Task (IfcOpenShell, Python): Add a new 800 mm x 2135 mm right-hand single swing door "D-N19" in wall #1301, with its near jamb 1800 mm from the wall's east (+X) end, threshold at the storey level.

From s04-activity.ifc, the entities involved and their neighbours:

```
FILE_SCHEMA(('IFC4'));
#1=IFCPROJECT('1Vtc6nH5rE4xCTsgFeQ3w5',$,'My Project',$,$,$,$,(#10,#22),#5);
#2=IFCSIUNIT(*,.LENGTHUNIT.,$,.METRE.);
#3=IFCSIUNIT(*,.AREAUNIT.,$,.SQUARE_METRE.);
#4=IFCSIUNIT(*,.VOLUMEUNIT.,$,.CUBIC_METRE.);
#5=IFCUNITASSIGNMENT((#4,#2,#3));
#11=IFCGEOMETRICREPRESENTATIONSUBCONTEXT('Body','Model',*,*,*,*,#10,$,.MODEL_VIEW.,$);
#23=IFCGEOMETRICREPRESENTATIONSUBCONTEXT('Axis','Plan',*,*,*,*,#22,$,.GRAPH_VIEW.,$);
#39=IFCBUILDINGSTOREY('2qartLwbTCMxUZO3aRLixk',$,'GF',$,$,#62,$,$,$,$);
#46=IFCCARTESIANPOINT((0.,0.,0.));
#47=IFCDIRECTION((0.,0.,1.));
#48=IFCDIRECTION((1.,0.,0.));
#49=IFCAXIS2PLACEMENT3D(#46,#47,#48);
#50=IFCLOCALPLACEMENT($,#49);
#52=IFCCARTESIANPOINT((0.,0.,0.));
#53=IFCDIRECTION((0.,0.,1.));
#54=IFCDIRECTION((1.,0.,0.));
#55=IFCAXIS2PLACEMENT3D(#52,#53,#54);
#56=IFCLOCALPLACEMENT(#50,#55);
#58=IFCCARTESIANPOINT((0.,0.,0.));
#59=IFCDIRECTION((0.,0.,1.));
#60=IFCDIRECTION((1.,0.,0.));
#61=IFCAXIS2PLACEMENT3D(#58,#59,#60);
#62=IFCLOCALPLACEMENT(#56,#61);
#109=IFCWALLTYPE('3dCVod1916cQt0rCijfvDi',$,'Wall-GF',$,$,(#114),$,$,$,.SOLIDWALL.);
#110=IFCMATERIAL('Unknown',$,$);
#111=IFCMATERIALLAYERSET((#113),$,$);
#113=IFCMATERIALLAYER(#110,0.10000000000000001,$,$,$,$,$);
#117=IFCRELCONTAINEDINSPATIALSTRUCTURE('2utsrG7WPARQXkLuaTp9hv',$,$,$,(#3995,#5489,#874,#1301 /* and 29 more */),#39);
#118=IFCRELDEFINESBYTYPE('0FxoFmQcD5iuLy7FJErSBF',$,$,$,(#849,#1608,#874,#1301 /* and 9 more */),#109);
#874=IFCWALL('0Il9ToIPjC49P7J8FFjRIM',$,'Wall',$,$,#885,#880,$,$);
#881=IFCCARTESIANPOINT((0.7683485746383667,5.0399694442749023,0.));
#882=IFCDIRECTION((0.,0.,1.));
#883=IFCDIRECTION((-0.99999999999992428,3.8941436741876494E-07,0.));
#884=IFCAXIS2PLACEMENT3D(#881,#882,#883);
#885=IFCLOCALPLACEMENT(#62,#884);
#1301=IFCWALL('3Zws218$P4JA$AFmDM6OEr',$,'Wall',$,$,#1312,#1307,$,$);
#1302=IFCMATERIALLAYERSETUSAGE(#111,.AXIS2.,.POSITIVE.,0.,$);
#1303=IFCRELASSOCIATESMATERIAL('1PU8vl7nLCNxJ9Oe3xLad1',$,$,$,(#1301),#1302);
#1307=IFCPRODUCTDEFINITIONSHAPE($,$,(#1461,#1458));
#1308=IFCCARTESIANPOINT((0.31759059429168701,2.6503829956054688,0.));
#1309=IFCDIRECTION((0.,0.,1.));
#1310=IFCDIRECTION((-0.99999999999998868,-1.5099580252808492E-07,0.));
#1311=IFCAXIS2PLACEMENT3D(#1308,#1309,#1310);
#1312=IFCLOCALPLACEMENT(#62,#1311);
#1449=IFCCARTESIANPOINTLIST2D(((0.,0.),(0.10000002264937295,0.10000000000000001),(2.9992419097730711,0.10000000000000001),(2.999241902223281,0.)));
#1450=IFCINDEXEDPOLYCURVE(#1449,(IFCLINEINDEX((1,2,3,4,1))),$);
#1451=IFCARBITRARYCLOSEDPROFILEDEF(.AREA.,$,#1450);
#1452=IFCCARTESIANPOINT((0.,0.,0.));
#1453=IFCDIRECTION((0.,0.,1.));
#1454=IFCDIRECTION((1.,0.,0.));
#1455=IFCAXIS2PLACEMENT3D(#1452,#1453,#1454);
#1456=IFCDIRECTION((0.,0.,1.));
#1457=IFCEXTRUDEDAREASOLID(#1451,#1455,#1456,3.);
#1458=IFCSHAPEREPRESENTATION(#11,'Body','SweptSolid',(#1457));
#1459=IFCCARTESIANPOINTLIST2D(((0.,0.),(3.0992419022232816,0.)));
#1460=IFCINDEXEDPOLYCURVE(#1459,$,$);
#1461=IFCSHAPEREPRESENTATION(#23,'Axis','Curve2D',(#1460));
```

```python
import numpy as np
import ifcopenshell
import ifcopenshell.api.feature
import ifcopenshell.api.geometry
import ifcopenshell.api.root
import ifcopenshell.api.spatial
import ifcopenshell.geom
import ifcopenshell.util.element
import ifcopenshell.util.placement
import ifcopenshell.util.representation
import ifcopenshell.util.shape
import ifcopenshell.util.unit

model = ifcopenshell.open("s04-activity.ifc")
unit_scale = ifcopenshell.util.unit.calculate_unit_scale(model)
settings = ifcopenshell.geom.settings()


def volume(element):
    """Net volume in cubic metres, openings subtracted."""
    shape = ifcopenshell.geom.create_shape(settings, element)
    return ifcopenshell.util.shape.get_volume(shape.geometry)


wall = model.by_guid("3Zws218$P4JA$AFmDM6OEr")
storey = ifcopenshell.util.element.get_container(wall, ifc_class="IfcBuildingStorey")
context = ifcopenshell.util.representation.get_context(model, "Model", "Body", "MODEL_VIEW")
before = volume(wall)

width, height, from_end, sill = 0.8, 2.135, 1.8, 0.0  # metres

# The wall runs along its own X axis, and the end named is its -X end.
wall_shape = ifcopenshell.geom.create_shape(settings, wall)
x, y, z = ifcopenshell.util.shape.get_vertices(wall_shape.geometry).T
start = x.min() + from_end
face, thickness = float(y.min()), float(y.max() - y.min())
wall_matrix = ifcopenshell.util.placement.get_local_placement(wall.ObjectPlacement)
level = ifcopenshell.util.placement.get_local_placement(storey.ObjectPlacement)[2, 3]


def in_wall(x, y):
    """Placement at x, y metres in the wall's axes, at sill height."""
    matrix = wall_matrix.copy()
    matrix[:, 3] = wall_matrix @ np.array([x / unit_scale, y / unit_scale, 0.0, 1.0])
    matrix[2, 3] = level + sill / unit_scale
    return matrix


# Opening: a box that overshoots both wall faces by 50 mm.
opening = ifcopenshell.api.root.create_entity(model, ifc_class="IfcOpeningElement", predefined_type="OPENING")
box = ifcopenshell.api.geometry.add_wall_representation(
    model, context=context, length=width, height=height, thickness=thickness + 0.1
)
ifcopenshell.api.geometry.assign_representation(model, product=opening, representation=box)
ifcopenshell.api.geometry.edit_object_placement(model, product=opening, matrix=in_wall(start, face - 0.05), is_si=False)
ifcopenshell.api.feature.add_feature(model, feature=opening, element=wall)

door = ifcopenshell.api.root.create_entity(model, ifc_class="IfcDoor", name="D-N19", predefined_type="DOOR")
door.OverallWidth, door.OverallHeight = width / unit_scale, height / unit_scale
door.OperationType = "SINGLE_SWING_RIGHT"
body = ifcopenshell.api.geometry.add_door_representation(
    model,
    context=context,
    overall_width=door.OverallWidth,
    overall_height=door.OverallHeight,
    operation_type="SINGLE_SWING_RIGHT",
    lining_properties={"LiningDepth": thickness / unit_scale, "ThresholdDepth": thickness / unit_scale},
)
ifcopenshell.api.geometry.assign_representation(model, product=door, representation=body)
ifcopenshell.api.spatial.assign_container(model, products=[door], relating_structure=storey)
ifcopenshell.api.feature.add_filling(model, opening=opening, element=door)

# The lining spans the wall, so the door starts at the wall face.
ifcopenshell.api.geometry.edit_object_placement(model, product=door, matrix=in_wall(start, face), is_si=False)

after = volume(wall)

print(f"wall volume {before:.3f} -> {after:.3f} m3")

model.write("s04-activity-out.ifc")
```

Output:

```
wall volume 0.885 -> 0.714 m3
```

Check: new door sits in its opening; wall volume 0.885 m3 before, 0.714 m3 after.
